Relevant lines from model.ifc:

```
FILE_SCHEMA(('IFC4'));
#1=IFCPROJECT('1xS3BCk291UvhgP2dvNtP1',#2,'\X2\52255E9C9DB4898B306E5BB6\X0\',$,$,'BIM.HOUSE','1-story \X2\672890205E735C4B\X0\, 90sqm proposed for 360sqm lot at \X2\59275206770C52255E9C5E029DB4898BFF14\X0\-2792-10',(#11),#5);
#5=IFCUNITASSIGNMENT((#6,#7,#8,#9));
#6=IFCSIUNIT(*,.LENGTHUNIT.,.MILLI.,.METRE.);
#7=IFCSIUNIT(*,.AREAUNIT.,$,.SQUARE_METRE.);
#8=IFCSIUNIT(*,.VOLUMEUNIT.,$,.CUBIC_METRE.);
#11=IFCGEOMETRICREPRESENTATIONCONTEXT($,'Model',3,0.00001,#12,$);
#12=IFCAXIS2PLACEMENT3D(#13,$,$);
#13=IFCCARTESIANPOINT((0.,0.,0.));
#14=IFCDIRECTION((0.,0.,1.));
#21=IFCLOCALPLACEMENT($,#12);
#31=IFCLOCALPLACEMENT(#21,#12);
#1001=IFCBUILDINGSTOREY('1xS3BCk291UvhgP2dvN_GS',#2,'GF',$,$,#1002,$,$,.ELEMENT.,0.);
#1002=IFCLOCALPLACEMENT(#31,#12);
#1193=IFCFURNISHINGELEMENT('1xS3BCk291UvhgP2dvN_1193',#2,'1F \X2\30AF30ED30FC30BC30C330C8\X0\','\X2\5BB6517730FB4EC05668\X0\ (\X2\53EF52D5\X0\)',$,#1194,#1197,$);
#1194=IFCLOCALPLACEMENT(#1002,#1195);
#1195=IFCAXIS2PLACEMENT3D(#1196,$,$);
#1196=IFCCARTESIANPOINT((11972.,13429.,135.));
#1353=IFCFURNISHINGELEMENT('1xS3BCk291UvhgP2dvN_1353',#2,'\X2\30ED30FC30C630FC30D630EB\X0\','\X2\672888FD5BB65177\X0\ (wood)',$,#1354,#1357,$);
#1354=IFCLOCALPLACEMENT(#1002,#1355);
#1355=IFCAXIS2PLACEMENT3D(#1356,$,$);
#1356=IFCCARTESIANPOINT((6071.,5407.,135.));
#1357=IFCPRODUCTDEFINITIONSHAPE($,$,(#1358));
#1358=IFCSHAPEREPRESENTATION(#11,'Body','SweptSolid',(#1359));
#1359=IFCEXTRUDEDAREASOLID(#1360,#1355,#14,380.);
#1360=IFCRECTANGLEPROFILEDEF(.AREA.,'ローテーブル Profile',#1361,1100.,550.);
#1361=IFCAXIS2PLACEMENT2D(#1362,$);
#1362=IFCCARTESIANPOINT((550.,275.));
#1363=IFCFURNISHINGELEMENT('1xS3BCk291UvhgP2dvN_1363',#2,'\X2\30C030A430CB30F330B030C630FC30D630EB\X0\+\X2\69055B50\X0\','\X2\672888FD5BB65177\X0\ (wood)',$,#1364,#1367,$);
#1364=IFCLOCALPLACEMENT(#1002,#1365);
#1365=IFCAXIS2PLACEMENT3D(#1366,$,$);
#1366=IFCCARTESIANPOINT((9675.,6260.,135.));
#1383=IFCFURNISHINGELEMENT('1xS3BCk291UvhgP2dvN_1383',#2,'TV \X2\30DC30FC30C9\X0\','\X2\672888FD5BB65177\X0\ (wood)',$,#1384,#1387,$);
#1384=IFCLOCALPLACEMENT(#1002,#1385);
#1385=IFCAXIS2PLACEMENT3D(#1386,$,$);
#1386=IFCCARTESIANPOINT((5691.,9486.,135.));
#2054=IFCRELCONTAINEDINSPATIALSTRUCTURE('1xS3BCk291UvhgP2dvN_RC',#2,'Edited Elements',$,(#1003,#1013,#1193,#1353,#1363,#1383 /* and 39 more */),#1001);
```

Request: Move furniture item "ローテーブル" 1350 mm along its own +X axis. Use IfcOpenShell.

```python
import ifcopenshell
import ifcopenshell.api.geometry
import ifcopenshell.util.placement
import ifcopenshell.util.unit

model = ifcopenshell.open("model.ifc")
unit_scale = ifcopenshell.util.unit.calculate_unit_scale(model)

item = model.by_guid("1xS3BCk291UvhgP2dvN_1353")
matrix = ifcopenshell.util.placement.get_local_placement(item.ObjectPlacement)
matrix[:3, 3] += matrix[:3, 0] * 1.35 / unit_scale
ifcopenshell.api.geometry.edit_object_placement(model, product=item, matrix=matrix, is_si=False)

print(ifcopenshell.util.placement.get_local_placement(item.ObjectPlacement).round(3) + 0.0)

model.write("model-out.ifc")
```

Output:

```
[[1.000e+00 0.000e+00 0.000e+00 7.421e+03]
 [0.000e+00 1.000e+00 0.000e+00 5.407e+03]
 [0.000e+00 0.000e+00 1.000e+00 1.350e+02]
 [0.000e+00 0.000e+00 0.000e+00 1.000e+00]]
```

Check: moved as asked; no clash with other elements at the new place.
